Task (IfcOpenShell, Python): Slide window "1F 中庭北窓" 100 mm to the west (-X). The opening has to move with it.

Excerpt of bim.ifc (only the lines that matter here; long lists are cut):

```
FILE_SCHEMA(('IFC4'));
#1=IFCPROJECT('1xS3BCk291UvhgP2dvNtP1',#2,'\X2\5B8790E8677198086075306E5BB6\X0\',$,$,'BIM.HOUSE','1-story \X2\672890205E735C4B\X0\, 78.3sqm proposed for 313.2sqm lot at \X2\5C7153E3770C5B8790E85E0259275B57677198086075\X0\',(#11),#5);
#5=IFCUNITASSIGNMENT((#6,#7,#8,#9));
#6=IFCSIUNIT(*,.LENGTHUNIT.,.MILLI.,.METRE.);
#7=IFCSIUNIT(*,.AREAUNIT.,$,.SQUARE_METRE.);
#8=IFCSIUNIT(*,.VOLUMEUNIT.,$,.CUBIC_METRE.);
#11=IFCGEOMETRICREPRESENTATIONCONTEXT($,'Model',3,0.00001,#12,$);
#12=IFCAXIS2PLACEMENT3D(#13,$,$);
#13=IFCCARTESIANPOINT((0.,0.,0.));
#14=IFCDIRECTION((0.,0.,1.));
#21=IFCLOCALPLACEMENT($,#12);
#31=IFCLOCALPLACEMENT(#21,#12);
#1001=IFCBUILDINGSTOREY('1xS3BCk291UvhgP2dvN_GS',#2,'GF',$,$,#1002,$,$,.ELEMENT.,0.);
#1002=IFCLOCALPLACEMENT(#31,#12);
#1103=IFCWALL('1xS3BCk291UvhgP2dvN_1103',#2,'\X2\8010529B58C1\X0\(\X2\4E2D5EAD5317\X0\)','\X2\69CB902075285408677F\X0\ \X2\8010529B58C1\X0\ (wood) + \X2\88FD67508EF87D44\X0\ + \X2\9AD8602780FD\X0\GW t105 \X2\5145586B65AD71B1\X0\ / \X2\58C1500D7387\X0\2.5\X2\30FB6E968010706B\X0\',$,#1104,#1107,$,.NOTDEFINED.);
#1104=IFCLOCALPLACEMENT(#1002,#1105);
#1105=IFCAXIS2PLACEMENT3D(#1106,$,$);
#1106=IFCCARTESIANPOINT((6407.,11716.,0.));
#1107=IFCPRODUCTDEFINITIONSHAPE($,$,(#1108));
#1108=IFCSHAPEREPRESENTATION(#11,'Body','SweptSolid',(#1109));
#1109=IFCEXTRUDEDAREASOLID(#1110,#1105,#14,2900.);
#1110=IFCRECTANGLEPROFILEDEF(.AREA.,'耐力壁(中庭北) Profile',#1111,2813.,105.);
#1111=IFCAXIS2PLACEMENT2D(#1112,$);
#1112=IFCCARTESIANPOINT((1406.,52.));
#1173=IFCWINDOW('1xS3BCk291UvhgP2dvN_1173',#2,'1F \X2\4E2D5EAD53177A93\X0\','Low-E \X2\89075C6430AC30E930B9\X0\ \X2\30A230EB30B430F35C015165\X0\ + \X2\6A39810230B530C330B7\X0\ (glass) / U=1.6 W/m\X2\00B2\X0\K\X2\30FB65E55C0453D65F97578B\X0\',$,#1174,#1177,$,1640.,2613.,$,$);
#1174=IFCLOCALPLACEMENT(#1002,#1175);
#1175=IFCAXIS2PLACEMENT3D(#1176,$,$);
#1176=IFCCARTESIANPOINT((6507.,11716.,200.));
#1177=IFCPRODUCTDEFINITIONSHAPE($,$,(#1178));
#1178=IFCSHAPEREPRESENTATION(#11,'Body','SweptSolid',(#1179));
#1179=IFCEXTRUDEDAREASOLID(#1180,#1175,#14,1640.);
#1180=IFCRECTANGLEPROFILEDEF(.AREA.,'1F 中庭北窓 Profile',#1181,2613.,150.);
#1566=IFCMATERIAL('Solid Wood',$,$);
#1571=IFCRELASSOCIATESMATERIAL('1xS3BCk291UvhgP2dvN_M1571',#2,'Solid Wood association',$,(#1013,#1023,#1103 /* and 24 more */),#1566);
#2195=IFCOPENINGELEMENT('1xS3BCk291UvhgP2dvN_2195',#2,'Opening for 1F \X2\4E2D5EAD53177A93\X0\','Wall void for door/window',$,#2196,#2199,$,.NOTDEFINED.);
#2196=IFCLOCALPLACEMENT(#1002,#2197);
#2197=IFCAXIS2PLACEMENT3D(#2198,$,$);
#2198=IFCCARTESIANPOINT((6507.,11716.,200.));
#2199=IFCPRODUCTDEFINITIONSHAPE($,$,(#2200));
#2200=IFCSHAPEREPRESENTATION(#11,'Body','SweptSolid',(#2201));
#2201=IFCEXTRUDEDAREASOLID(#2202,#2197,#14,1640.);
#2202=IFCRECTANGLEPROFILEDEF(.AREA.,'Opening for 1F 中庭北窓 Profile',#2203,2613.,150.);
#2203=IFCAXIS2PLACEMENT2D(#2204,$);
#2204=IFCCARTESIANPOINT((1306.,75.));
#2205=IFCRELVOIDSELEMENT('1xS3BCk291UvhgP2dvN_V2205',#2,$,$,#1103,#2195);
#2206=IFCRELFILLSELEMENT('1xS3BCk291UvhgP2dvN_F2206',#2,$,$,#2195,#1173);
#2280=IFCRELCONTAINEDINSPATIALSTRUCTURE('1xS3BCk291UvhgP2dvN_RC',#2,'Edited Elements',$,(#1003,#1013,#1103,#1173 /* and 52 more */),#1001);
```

```python
import ifcopenshell
import ifcopenshell.api.geometry
import ifcopenshell.util.placement

model = ifcopenshell.open("bim.ifc")

window = model.by_guid("1xS3BCk291UvhgP2dvN_1173")
opening = window.FillsVoids[0].RelatingOpeningElement
wall = opening.VoidsElements[0].RelatingBuildingElement

wall_matrix = ifcopenshell.util.placement.get_local_placement(wall.ObjectPlacement)
shift = wall_matrix[:3, 0] * -100.0
before = ifcopenshell.util.placement.get_local_placement(window.ObjectPlacement)[:3, 3].copy()

# The window is not placed relative to its opening, so move both.
for product in (opening, window):
    matrix = ifcopenshell.util.placement.get_local_placement(product.ObjectPlacement)
    matrix[:3, 3] += shift
    ifcopenshell.api.geometry.edit_object_placement(model, product=product, matrix=matrix, is_si=False)

after = ifcopenshell.util.placement.get_local_placement(window.ObjectPlacement)[:3, 3]
print("window moved by", (after - before).round(3) + 0.0)

model.write("bim_updated.ifc")
```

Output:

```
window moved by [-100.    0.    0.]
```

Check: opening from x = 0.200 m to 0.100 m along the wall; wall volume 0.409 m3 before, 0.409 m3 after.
